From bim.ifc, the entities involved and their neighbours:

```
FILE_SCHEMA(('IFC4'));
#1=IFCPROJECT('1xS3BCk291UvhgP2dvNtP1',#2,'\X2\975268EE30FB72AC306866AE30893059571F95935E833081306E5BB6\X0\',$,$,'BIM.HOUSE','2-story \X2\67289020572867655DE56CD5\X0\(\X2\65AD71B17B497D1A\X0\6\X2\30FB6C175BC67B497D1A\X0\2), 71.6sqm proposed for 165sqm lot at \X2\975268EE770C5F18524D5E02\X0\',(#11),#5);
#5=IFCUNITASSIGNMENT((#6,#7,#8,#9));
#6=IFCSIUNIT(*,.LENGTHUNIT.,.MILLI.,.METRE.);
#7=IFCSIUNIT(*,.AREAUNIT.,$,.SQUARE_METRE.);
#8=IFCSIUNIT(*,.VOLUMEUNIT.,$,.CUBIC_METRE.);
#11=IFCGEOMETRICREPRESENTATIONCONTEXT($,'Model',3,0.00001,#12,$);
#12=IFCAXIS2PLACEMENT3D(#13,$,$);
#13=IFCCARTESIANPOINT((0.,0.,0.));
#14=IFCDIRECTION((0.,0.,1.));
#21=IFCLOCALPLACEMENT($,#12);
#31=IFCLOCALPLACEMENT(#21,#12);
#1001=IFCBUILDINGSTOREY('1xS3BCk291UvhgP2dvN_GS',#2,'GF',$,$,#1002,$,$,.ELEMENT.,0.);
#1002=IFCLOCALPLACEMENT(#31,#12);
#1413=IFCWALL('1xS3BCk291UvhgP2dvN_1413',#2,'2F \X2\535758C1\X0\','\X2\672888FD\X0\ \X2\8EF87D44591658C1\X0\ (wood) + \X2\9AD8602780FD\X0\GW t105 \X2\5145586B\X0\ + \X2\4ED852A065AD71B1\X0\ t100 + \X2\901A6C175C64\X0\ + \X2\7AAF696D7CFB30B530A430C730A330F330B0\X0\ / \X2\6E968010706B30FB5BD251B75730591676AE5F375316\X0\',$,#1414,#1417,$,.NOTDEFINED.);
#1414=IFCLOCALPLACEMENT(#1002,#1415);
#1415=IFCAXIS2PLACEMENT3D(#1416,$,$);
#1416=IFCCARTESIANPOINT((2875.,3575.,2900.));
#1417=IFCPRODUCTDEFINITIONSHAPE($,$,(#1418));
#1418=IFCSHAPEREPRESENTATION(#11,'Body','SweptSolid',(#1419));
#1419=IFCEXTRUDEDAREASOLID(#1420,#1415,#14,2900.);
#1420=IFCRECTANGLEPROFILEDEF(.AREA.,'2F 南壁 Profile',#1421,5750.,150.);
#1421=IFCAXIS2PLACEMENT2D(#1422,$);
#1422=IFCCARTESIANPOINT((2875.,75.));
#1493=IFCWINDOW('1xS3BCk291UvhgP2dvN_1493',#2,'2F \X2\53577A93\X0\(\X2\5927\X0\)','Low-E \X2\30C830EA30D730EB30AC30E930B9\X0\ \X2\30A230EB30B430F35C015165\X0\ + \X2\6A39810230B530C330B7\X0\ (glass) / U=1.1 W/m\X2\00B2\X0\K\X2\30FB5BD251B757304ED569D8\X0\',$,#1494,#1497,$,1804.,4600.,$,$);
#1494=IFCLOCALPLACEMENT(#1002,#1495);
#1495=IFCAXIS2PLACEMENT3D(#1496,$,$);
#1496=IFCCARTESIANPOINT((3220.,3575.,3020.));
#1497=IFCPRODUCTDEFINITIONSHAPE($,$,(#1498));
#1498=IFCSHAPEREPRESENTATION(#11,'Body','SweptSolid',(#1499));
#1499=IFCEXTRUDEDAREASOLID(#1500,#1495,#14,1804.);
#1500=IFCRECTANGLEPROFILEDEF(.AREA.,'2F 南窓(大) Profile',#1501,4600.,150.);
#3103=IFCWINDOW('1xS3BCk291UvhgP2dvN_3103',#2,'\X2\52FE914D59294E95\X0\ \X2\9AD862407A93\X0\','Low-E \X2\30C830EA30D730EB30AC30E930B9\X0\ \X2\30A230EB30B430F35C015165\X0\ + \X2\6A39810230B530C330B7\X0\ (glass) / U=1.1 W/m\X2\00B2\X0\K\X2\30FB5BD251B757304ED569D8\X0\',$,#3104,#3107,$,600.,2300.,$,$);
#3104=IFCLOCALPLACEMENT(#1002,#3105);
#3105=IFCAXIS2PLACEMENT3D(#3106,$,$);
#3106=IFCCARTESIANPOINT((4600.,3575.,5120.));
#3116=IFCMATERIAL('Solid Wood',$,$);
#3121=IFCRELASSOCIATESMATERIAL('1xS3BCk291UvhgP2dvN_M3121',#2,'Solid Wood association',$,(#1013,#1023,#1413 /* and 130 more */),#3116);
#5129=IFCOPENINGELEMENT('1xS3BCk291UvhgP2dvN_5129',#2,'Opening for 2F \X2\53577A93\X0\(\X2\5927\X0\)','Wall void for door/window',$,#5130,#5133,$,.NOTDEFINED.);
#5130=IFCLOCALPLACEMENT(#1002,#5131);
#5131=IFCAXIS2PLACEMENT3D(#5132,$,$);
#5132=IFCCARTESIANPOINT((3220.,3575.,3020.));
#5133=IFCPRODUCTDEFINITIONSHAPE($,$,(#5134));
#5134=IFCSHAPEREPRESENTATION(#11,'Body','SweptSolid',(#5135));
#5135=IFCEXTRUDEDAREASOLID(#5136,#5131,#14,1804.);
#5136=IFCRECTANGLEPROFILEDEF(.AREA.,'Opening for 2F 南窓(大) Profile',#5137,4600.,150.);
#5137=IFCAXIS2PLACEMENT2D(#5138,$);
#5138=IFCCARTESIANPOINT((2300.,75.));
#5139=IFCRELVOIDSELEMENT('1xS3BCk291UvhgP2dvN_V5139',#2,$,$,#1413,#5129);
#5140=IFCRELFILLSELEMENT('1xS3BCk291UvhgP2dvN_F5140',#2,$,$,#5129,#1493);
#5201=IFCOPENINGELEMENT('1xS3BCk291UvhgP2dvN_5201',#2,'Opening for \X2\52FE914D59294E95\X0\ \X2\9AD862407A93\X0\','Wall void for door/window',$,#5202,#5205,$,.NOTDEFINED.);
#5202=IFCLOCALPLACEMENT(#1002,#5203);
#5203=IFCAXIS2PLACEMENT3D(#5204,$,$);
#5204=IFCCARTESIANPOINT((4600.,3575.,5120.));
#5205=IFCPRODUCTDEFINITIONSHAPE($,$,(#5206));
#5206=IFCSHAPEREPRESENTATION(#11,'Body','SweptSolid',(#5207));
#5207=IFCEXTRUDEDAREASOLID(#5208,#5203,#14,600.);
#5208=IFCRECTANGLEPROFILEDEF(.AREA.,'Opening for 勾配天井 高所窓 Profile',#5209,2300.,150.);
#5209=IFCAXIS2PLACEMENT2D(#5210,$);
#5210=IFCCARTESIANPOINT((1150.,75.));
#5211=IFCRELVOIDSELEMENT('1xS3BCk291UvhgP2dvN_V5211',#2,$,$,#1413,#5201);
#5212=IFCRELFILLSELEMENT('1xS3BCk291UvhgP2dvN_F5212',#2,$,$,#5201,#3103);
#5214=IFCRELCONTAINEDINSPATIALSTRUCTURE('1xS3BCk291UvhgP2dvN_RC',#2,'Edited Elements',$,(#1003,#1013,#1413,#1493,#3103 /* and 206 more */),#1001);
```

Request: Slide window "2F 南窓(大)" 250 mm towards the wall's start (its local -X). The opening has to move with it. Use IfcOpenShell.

```python
import ifcopenshell
import ifcopenshell.api.geometry
import ifcopenshell.util.placement

model = ifcopenshell.open("bim.ifc")

window = model.by_guid("1xS3BCk291UvhgP2dvN_1493")
opening = window.FillsVoids[0].RelatingOpeningElement
wall = opening.VoidsElements[0].RelatingBuildingElement

wall_matrix = ifcopenshell.util.placement.get_local_placement(wall.ObjectPlacement)
shift = wall_matrix[:3, 0] * -250.0
before = ifcopenshell.util.placement.get_local_placement(window.ObjectPlacement)[:3, 3].copy()

# The window is not placed relative to its opening, so move both.
for product in (opening, window):
    matrix = ifcopenshell.util.placement.get_local_placement(product.ObjectPlacement)
    matrix[:3, 3] += shift
    ifcopenshell.api.geometry.edit_object_placement(model, product=product, matrix=matrix, is_si=False)

after = ifcopenshell.util.placement.get_local_placement(window.ObjectPlacement)[:3, 3]
print("window moved by", (after - before).round(3) + 0.0)

model.write("bim-out.ifc")
```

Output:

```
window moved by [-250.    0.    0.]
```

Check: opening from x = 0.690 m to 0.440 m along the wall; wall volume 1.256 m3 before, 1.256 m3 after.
